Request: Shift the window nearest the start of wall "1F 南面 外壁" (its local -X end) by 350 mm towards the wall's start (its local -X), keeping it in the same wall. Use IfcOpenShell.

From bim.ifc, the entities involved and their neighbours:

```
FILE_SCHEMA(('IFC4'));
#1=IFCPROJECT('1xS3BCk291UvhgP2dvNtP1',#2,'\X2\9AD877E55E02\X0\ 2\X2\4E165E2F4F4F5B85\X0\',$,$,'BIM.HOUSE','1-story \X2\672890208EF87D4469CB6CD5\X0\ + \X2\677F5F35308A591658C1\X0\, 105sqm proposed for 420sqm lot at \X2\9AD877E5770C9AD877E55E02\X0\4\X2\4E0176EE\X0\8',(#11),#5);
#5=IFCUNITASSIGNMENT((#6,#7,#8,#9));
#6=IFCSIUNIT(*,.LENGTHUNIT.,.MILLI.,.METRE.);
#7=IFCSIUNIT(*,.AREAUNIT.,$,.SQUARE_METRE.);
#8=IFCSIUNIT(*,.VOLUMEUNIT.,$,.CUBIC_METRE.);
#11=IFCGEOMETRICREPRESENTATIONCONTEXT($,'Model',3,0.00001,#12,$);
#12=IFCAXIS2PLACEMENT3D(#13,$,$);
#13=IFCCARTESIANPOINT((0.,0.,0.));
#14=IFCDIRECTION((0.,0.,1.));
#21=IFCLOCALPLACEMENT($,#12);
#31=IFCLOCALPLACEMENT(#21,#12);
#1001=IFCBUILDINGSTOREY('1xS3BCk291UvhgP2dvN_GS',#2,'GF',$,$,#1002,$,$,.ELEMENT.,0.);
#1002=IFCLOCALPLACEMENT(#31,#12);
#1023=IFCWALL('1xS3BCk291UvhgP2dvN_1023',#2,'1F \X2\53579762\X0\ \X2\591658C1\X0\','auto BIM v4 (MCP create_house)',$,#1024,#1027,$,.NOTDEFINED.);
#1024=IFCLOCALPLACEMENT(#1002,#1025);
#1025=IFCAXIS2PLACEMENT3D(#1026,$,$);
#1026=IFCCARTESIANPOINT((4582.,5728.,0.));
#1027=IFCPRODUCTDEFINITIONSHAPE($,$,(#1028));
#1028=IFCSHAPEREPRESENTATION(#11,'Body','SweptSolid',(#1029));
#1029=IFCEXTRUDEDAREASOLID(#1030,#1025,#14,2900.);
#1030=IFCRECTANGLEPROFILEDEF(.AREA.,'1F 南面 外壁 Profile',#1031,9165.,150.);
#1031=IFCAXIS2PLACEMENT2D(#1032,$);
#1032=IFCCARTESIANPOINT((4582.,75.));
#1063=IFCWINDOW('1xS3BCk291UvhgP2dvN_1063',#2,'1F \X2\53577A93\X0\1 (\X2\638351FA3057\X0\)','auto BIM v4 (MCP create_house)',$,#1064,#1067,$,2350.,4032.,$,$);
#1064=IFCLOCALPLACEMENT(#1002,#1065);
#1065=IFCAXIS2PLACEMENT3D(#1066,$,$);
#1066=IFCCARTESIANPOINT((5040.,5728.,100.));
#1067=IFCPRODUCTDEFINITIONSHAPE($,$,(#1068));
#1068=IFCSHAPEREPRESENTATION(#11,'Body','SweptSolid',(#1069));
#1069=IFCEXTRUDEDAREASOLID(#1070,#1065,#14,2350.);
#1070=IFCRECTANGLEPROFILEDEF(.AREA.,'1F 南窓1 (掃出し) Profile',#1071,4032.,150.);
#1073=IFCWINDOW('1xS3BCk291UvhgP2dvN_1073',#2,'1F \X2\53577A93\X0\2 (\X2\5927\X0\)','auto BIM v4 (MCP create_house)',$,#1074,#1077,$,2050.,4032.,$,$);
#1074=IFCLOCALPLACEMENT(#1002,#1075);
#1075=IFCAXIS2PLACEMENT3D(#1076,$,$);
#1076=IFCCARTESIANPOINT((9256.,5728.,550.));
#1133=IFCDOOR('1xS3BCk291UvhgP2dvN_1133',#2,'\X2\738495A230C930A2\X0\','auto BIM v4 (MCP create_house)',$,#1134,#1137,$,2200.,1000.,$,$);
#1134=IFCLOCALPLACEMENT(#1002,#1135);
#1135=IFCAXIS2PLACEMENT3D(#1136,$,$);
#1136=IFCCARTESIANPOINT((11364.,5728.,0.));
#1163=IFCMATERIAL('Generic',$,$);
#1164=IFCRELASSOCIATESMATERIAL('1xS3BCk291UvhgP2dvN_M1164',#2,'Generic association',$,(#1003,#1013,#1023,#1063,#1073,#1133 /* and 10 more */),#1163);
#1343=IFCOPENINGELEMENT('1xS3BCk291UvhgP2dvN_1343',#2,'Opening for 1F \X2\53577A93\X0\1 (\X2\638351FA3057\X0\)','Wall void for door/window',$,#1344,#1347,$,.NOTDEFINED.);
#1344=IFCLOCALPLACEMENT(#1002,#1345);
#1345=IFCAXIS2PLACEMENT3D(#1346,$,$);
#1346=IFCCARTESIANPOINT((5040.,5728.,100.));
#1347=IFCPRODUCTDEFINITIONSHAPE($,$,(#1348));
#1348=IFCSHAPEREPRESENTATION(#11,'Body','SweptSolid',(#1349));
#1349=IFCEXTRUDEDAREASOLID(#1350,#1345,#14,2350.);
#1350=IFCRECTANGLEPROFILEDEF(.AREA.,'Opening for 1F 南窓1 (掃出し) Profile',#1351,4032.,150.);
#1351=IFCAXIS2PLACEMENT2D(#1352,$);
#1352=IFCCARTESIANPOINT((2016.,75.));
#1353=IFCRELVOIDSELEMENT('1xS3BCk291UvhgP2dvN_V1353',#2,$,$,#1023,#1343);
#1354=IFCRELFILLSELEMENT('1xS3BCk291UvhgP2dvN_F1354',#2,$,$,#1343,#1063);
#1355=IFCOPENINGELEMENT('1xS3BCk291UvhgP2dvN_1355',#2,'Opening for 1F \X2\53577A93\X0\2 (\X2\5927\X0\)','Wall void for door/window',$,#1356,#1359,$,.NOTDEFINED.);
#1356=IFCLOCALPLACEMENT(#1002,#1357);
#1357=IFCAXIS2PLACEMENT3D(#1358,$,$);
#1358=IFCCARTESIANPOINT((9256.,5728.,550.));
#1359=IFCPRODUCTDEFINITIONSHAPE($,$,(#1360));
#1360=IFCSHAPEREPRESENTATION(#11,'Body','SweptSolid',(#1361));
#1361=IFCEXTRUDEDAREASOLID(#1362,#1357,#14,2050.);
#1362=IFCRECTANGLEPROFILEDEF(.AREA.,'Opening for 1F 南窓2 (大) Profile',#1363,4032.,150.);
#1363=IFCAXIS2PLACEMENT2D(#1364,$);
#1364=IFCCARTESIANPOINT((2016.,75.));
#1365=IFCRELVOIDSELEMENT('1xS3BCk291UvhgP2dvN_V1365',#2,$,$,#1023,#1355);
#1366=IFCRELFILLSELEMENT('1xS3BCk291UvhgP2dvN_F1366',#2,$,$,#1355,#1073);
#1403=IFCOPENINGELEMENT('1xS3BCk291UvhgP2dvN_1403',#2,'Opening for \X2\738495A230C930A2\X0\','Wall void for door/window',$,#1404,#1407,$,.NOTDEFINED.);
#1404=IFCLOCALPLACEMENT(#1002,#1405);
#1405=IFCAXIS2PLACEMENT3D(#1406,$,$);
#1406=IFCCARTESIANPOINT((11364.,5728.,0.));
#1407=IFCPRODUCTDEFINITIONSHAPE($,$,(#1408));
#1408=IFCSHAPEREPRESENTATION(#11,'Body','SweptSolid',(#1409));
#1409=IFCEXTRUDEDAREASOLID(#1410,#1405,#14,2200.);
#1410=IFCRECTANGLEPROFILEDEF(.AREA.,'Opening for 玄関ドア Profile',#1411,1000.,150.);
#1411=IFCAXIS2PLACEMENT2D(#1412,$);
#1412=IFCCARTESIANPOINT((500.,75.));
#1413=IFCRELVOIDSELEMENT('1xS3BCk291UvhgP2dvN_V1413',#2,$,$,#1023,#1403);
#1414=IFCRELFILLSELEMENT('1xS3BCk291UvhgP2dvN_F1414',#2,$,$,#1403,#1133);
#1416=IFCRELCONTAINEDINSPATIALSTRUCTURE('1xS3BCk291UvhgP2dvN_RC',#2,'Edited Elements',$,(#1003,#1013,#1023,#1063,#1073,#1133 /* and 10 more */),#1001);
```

```python
import ifcopenshell
import ifcopenshell.api.geometry
import ifcopenshell.util.placement

model = ifcopenshell.open("bim.ifc")

window = model.by_guid("1xS3BCk291UvhgP2dvN_1063")
opening = window.FillsVoids[0].RelatingOpeningElement
wall = opening.VoidsElements[0].RelatingBuildingElement

wall_matrix = ifcopenshell.util.placement.get_local_placement(wall.ObjectPlacement)
shift = wall_matrix[:3, 0] * -350.0
before = ifcopenshell.util.placement.get_local_placement(window.ObjectPlacement)[:3, 3].copy()

# The window is not placed relative to its opening, so move both.
for product in (opening, window):
    matrix = ifcopenshell.util.placement.get_local_placement(product.ObjectPlacement)
    matrix[:3, 3] += shift
    ifcopenshell.api.geometry.edit_object_placement(model, product=product, matrix=matrix, is_si=False)

after = ifcopenshell.util.placement.get_local_placement(window.ObjectPlacement)[:3, 3]
print("window moved by", (after - before).round(3) + 0.0)

model.write("bim_updated.ifc")
```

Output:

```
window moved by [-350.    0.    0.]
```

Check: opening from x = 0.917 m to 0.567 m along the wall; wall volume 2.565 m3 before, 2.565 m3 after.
